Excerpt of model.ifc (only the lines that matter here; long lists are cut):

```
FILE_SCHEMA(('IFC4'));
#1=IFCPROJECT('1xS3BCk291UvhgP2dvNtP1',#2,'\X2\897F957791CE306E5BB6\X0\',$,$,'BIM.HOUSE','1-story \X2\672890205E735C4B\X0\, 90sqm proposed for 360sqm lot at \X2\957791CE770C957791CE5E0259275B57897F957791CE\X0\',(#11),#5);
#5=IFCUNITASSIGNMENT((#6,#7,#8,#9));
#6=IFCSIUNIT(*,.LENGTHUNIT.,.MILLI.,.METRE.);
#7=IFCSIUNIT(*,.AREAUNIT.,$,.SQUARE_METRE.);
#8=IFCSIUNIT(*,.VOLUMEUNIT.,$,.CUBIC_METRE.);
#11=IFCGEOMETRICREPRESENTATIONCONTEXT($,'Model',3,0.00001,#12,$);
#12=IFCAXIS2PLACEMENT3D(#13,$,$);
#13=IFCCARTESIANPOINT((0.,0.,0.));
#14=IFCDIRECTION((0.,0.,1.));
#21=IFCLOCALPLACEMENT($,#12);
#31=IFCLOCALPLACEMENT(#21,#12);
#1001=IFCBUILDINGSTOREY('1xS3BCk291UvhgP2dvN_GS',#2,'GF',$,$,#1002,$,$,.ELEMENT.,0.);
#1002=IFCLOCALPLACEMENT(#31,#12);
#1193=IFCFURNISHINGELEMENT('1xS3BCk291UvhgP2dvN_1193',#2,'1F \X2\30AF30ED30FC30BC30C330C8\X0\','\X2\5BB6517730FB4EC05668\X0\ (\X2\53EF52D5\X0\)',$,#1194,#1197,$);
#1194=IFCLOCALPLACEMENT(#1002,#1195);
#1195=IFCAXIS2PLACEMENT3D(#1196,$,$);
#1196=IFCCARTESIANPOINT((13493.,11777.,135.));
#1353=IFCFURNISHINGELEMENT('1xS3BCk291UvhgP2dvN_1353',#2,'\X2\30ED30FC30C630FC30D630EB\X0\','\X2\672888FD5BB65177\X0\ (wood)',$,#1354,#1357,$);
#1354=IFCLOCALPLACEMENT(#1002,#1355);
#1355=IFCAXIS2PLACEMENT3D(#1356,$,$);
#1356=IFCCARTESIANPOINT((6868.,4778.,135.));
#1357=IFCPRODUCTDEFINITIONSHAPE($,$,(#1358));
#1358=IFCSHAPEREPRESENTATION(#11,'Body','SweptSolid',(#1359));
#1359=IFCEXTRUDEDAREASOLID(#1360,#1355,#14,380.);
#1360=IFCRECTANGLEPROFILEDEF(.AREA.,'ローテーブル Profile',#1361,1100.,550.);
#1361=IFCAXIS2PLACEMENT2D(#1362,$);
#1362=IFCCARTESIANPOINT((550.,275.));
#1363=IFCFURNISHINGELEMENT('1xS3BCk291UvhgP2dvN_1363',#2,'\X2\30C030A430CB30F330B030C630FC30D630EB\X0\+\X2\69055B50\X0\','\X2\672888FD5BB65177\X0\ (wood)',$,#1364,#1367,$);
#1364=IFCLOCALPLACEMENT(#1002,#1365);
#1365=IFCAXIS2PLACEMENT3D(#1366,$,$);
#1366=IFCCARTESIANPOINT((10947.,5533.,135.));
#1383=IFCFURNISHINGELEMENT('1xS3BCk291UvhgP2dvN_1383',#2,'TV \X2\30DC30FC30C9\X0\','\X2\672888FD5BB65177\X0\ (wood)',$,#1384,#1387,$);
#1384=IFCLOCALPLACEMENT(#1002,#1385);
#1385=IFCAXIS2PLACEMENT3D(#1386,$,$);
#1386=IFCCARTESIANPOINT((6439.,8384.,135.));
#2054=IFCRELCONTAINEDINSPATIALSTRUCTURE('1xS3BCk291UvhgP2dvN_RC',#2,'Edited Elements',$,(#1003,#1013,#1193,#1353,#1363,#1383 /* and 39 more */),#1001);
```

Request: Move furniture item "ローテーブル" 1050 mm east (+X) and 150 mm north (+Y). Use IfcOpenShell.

```python
import ifcopenshell
import ifcopenshell.api.geometry
import ifcopenshell.util.placement

model = ifcopenshell.open("model.ifc")

item = model.by_guid("1xS3BCk291UvhgP2dvN_1353")
matrix = ifcopenshell.util.placement.get_local_placement(item.ObjectPlacement)
matrix[0, 3] += 1050.0
matrix[1, 3] += 150.0
ifcopenshell.api.geometry.edit_object_placement(model, product=item, matrix=matrix, is_si=False)

print(ifcopenshell.util.placement.get_local_placement(item.ObjectPlacement).round(3) + 0.0)

model.write("model_edited.ifc")
```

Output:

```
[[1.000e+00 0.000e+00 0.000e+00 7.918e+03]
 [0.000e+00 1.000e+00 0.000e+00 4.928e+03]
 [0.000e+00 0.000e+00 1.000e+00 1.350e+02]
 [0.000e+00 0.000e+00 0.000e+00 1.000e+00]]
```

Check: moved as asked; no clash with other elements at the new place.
